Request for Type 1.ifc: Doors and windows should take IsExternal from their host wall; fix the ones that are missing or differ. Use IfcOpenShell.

First a look at what the model holds.

```python
import ifcopenshell
import ifcopenshell.util.element

model = ifcopenshell.open("Type 1.ifc")
print(model.schema)
seen = {}
for e in model.by_type("IfcDoor") + model.by_type("IfcWindow"):
    if not e.FillsVoids:
        continue
    host = e.FillsVoids[0].RelatingOpeningElement.VoidsElements[0].RelatingBuildingElement
    own = ifcopenshell.util.element.get_pset(e, f"Pset_{e.is_a()[3:].removesuffix('StandardCase')}Common", "IsExternal")
    wall = ifcopenshell.util.element.get_pset(host, "Pset_WallCommon", "IsExternal")
    seen[e.is_a(), own, wall] = seen.get((e.is_a(), own, wall), 0) + 1
for (cls, own, wall), count in sorted(seen.items(), key=str):
    print(count, cls, "IsExternal:", own, "| host wall:", wall)
```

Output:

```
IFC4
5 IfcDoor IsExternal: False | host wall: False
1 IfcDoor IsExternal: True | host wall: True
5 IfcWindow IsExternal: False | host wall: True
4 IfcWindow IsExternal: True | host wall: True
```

```python
import ifcopenshell
import ifcopenshell.api.pset
import ifcopenshell.util.element

model = ifcopenshell.open("Type 1.ifc")

count = 0
for ifc_class, pset_name in (("IfcDoor", "Pset_DoorCommon"), ("IfcWindow", "Pset_WindowCommon")):
    for e in model.by_type(ifc_class):
        if not e.FillsVoids:
            continue
        host = e.FillsVoids[0].RelatingOpeningElement.VoidsElements[0].RelatingBuildingElement
        external = ifcopenshell.util.element.get_pset(host, "Pset_WallCommon", "IsExternal")
        if external is None or ifcopenshell.util.element.get_pset(e, pset_name, "IsExternal") == external:
            continue
        pset = ifcopenshell.api.pset.add_pset(model, product=e, name=pset_name)
        ifcopenshell.api.pset.edit_pset(model, pset=pset, properties={"IsExternal": external})
        count += 1

print(count, "updated")

model.write("Type 1_v2.ifc")
```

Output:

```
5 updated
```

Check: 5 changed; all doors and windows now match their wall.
